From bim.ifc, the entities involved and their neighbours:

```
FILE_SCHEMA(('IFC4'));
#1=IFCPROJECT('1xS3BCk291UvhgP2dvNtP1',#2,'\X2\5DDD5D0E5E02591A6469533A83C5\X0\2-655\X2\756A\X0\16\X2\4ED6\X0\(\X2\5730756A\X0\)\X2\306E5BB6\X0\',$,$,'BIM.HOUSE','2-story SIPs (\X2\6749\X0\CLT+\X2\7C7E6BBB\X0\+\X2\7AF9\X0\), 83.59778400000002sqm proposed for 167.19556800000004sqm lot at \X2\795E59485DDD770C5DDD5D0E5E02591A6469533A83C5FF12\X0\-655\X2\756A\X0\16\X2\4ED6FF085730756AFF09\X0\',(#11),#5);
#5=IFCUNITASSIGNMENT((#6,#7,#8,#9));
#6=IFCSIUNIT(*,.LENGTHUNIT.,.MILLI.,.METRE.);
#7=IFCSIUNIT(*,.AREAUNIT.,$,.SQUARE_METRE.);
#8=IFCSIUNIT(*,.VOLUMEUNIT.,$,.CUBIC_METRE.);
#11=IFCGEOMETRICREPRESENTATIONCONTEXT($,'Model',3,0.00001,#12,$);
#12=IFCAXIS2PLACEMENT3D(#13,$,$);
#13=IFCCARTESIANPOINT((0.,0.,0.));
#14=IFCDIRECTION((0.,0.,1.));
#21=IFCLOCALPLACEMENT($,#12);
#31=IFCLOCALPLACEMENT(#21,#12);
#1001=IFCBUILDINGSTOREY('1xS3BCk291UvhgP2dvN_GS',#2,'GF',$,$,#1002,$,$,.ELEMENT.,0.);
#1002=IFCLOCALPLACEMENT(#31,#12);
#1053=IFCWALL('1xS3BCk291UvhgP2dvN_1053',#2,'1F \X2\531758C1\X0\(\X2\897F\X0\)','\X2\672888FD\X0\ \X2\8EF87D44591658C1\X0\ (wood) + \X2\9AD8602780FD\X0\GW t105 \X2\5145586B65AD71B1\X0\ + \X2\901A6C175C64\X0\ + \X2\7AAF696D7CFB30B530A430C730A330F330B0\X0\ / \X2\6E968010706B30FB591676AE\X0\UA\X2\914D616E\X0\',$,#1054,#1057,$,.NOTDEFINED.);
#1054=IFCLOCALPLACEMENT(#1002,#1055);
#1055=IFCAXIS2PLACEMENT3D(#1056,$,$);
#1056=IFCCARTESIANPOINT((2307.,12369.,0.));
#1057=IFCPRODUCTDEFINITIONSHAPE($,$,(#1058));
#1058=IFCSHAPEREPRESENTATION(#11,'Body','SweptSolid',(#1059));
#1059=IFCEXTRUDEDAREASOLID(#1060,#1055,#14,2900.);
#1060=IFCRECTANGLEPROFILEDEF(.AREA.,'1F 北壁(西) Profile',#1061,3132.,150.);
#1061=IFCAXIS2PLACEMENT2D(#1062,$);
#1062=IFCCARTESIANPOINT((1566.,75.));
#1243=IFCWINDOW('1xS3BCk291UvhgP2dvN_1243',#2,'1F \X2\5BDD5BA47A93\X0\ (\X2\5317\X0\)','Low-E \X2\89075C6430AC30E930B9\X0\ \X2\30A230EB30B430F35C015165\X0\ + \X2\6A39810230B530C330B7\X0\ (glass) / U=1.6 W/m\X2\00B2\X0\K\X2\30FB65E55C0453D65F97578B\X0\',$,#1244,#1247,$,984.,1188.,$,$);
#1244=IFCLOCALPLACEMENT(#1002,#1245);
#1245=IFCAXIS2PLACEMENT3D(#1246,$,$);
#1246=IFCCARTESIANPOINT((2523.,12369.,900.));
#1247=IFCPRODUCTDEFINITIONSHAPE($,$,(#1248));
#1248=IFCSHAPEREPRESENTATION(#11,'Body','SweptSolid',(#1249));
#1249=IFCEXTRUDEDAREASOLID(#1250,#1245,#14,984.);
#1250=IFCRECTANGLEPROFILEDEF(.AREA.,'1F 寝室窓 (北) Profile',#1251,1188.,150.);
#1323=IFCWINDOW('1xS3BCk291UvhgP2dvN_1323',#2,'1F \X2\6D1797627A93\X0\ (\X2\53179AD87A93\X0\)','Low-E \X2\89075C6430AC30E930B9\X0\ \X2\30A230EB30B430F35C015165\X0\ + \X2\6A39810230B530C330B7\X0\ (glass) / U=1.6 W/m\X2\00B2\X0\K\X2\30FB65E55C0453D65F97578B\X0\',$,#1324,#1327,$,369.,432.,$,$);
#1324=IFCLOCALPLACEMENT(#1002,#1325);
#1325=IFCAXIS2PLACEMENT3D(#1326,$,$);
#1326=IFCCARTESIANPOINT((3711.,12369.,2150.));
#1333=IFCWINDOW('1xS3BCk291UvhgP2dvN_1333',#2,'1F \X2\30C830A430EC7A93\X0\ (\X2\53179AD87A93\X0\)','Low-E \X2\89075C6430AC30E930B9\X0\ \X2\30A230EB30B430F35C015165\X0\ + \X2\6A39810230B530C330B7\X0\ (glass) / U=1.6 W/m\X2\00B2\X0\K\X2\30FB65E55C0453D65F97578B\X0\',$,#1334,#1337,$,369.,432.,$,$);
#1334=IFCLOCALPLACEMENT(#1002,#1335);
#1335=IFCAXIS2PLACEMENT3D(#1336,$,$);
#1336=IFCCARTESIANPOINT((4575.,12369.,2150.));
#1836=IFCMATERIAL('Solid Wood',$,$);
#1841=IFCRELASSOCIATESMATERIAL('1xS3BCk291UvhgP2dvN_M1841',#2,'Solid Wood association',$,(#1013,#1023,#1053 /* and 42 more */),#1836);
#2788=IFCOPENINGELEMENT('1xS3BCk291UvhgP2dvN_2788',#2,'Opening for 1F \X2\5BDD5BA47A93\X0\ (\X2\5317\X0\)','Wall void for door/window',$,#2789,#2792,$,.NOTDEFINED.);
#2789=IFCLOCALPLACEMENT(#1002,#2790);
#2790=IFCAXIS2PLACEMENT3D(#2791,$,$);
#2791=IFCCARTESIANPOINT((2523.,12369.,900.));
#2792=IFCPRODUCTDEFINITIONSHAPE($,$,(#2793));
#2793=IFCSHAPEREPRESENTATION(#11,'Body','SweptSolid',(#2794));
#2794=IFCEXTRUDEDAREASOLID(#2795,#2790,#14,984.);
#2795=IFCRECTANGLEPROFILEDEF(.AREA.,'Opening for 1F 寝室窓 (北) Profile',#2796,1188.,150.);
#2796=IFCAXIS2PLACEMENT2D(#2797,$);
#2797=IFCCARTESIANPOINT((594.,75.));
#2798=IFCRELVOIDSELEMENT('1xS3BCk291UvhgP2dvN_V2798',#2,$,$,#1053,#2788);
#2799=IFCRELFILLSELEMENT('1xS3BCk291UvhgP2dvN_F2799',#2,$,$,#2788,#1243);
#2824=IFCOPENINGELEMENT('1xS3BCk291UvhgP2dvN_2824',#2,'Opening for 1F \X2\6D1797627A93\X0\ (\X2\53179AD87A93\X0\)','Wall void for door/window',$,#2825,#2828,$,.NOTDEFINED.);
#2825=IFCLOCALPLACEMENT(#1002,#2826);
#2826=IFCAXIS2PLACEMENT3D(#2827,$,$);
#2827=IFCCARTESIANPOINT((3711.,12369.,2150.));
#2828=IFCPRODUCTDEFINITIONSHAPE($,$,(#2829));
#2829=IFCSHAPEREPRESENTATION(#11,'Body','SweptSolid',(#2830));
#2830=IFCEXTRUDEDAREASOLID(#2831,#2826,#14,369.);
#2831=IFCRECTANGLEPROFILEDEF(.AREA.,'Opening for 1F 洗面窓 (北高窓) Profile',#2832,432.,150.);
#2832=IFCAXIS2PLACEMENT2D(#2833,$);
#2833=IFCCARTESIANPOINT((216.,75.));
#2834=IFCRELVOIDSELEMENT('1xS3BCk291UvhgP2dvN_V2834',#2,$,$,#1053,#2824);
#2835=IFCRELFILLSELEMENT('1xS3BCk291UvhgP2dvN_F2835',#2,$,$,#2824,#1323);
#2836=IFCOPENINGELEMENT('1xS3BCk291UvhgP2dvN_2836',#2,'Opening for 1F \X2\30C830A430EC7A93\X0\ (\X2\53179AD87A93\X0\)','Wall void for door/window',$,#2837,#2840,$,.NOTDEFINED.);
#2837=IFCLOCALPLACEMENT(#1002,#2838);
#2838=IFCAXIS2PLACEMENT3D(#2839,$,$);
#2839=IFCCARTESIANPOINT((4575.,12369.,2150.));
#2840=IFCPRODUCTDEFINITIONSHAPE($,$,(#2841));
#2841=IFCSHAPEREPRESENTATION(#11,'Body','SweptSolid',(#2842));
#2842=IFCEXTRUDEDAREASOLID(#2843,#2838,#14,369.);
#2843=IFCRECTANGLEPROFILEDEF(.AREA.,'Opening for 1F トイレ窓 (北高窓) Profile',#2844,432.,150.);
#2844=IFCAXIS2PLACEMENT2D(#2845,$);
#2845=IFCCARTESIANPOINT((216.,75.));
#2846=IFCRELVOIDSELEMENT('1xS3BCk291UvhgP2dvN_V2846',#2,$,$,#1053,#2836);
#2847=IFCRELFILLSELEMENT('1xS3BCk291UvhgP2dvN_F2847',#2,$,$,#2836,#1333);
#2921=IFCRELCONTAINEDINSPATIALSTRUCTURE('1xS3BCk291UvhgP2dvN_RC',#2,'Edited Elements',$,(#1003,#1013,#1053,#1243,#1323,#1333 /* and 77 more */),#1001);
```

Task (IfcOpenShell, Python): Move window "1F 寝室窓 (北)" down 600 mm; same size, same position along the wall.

```python
import numpy as np
import ifcopenshell
import ifcopenshell.api.geometry
import ifcopenshell.util.placement
import ifcopenshell.util.unit

model = ifcopenshell.open("bim.ifc")
unit_scale = ifcopenshell.util.unit.calculate_unit_scale(model)

window = model.by_id(1243)
opening = window.FillsVoids[0].RelatingOpeningElement
dz = -0.6 / unit_scale

shift = np.array([0.0, 0.0, dz])
# The window is not placed relative to its opening, so move both.
for product in (opening, window):
    matrix = ifcopenshell.util.placement.get_local_placement(product.ObjectPlacement)
    matrix[:3, 3] += shift
    ifcopenshell.api.geometry.edit_object_placement(model, product=product, matrix=matrix, is_si=False)

print(f"moved by {dz * unit_scale:+.3f} m")

model.write("bim_v2.ifc")
```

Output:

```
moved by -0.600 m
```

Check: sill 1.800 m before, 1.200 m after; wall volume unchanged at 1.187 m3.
